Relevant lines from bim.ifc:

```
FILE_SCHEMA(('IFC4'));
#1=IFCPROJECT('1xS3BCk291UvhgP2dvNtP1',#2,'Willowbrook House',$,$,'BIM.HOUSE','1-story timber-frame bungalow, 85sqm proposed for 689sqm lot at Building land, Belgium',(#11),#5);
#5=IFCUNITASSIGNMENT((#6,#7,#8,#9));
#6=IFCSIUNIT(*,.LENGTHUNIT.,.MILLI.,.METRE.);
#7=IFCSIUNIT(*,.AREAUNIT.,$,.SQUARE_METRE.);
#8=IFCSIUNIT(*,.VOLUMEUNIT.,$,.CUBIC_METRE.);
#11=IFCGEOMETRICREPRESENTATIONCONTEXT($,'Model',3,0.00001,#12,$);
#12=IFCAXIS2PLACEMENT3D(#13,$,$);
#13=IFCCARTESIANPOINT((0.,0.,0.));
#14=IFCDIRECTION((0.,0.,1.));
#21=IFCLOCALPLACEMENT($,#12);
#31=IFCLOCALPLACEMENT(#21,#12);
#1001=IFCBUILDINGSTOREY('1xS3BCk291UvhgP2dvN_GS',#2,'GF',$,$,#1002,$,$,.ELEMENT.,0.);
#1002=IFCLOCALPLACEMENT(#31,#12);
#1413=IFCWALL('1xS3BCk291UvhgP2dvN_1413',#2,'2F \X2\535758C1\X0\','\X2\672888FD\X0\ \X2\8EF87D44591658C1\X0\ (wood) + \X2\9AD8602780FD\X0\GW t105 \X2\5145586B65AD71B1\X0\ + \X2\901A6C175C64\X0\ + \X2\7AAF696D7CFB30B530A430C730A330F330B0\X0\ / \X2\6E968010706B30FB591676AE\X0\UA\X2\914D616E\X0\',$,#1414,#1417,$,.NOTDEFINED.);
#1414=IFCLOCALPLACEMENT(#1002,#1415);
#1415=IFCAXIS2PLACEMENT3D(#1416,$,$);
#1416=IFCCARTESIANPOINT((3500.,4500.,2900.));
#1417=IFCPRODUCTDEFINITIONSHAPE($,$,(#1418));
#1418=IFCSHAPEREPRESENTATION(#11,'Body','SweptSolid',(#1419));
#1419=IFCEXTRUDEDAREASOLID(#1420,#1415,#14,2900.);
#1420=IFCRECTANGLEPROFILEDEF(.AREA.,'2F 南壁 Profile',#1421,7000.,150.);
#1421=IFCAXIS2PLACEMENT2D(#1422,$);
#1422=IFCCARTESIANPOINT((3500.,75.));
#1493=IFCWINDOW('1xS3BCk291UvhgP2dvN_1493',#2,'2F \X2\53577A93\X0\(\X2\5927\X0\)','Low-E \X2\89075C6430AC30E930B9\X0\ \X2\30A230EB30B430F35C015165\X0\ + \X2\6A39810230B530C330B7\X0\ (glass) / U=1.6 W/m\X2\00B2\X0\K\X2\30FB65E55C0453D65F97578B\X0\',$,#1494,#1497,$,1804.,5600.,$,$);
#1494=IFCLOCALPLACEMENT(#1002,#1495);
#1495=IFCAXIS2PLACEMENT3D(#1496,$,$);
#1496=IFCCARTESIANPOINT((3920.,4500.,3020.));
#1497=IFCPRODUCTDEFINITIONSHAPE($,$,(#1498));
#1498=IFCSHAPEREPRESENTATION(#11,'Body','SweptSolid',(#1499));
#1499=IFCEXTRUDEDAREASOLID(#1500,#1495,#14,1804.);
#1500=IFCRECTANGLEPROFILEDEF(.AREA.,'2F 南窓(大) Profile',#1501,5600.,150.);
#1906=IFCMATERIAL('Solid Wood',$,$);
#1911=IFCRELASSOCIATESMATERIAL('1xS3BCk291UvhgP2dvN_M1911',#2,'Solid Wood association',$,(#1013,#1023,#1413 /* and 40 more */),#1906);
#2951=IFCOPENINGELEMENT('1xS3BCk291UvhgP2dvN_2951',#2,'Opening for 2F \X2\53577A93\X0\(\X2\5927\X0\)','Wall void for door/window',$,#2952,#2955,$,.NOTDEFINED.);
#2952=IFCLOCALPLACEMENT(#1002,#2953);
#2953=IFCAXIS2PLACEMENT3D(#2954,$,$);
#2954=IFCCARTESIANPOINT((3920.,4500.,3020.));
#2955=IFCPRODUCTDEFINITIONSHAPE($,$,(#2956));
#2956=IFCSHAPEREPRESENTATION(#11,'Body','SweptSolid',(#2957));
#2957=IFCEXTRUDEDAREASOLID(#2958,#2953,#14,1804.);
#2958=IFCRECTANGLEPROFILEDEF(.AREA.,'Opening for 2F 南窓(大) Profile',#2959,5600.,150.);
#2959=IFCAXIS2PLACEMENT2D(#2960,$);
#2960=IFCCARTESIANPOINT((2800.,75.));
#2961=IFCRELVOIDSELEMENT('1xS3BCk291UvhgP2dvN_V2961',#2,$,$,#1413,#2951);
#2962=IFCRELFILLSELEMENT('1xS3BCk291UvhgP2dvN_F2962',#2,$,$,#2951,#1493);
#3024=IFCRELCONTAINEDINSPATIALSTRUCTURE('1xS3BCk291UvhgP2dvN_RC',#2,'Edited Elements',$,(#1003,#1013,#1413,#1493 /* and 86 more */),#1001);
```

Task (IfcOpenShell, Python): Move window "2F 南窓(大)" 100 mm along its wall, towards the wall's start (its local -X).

```python
import ifcopenshell
import ifcopenshell.api.geometry
import ifcopenshell.util.placement

model = ifcopenshell.open("bim.ifc")

window = model.by_guid("1xS3BCk291UvhgP2dvN_1493")
opening = window.FillsVoids[0].RelatingOpeningElement
wall = opening.VoidsElements[0].RelatingBuildingElement

wall_matrix = ifcopenshell.util.placement.get_local_placement(wall.ObjectPlacement)
shift = wall_matrix[:3, 0] * -100.0
before = ifcopenshell.util.placement.get_local_placement(window.ObjectPlacement)[:3, 3].copy()

# The window is not placed relative to its opening, so move both.
for product in (opening, window):
    matrix = ifcopenshell.util.placement.get_local_placement(product.ObjectPlacement)
    matrix[:3, 3] += shift
    ifcopenshell.api.geometry.edit_object_placement(model, product=product, matrix=matrix, is_si=False)

after = ifcopenshell.util.placement.get_local_placement(window.ObjectPlacement)[:3, 3]
print("window moved by", (after - before).round(3) + 0.0)

model.write("bim_updated.ifc")
```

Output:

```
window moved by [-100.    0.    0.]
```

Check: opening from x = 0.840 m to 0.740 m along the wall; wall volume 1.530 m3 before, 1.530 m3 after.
